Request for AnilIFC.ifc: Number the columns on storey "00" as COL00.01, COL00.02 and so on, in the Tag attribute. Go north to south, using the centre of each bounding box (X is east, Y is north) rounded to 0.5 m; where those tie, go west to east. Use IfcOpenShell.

First a look at what the model holds.

```python
import ifcopenshell
import ifcopenshell.util.element
import ifcopenshell.util.placement

model = ifcopenshell.open("AnilIFC.ifc")
print(model.schema)
storey = next(s for s in model.by_type("IfcBuildingStorey") if s.Name == "00")
columns = [e for e in ifcopenshell.util.element.get_decomposition(storey) if e.is_a("IfcColumn")]
for e in sorted(columns, key=lambda e: e.id()):
    origin = ifcopenshell.util.placement.get_local_placement(e.ObjectPlacement)[:3, 3]
    print(e.id(), e.Tag, e.Name, origin.round(2) + 0.0, sep=" | ")
```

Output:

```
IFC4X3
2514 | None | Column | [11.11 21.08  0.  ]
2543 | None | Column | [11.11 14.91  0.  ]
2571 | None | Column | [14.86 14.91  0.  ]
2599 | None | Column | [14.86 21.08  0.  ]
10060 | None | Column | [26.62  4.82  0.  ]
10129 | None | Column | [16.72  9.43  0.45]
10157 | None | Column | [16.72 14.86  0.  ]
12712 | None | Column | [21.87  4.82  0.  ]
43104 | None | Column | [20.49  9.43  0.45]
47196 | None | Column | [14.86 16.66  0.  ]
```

```python
import ifcopenshell
import ifcopenshell.geom
import ifcopenshell.util.element
import ifcopenshell.util.shape

model = ifcopenshell.open("AnilIFC.ifc")
settings = ifcopenshell.geom.settings()
settings.set("use-world-coords", True)


def centre(element):
    shape = ifcopenshell.geom.create_shape(settings, element)
    return ifcopenshell.util.shape.get_bbox_centroid(shape.geometry)


storey = next(s for s in model.by_type("IfcBuildingStorey") if s.Name == "00")
columns = [e for e in ifcopenshell.util.element.get_decomposition(storey) if e.is_a("IfcColumn")]

# Insertion points can sit at a corner or the storey origin, so sort by the geometry (in metres).
centres = {e: centre(e) for e in columns}
columns.sort(key=lambda e: (-round(centres[e][1] / 0.5), centres[e][0]))

for i, e in enumerate(columns, start=1):
    number = f"COL00.{i:02d}"
    e.Tag = number
    print(e.id(), number)

model.write("AnilIFC-out.ifc")
```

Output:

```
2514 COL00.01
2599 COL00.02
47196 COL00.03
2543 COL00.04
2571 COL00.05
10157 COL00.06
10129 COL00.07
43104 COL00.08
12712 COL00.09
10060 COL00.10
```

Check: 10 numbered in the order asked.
